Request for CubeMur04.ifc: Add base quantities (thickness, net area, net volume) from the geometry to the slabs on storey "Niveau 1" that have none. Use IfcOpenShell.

First a look at what the model holds.

```python
import ifcopenshell
import ifcopenshell.util.element
import ifcopenshell.util.unit

model = ifcopenshell.open("CubeMur04.ifc")
print(model.schema)
for unit_type in ("LENGTHUNIT", "AREAUNIT", "VOLUMEUNIT"):
    print(unit_type, ifcopenshell.util.unit.calculate_unit_scale(model, unit_type))
storey = next(s for s in model.by_type("IfcBuildingStorey") if s.Name == "Niveau 1")
slabs = [e for e in ifcopenshell.util.element.get_decomposition(storey) if e.is_a("IfcSlab")]
for e in sorted(slabs, key=lambda e: e.id()):
    print(e.id(), e.is_a(), e.Name, list(ifcopenshell.util.element.get_psets(e, qtos_only=True)), sep=" | ")
```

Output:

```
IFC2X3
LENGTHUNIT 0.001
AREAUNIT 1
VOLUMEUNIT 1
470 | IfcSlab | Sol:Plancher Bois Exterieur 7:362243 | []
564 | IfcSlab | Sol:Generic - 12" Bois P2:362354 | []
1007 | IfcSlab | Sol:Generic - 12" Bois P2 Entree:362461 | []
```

```python
import ifcopenshell
import ifcopenshell.api.pset
import ifcopenshell.geom
import ifcopenshell.util.element
import ifcopenshell.util.shape
import ifcopenshell.util.unit

model = ifcopenshell.open("CubeMur04.ifc")
unit_scale = ifcopenshell.util.unit.calculate_unit_scale(model)
area_scale = ifcopenshell.util.unit.calculate_unit_scale(model, "AREAUNIT")
volume_scale = ifcopenshell.util.unit.calculate_unit_scale(model, "VOLUMEUNIT")
settings = ifcopenshell.geom.settings()

storey = next(s for s in model.by_type("IfcBuildingStorey") if s.Name == "Niveau 1")
slabs = [e for e in ifcopenshell.util.element.get_decomposition(storey) if e.is_a("IfcSlab")]

for e in sorted(slabs, key=lambda e: e.id()):
    if ifcopenshell.util.element.get_psets(e, qtos_only=True, should_inherit=False):
        continue
    # Geometry comes back in metres, in the element's own axes.
    shape = ifcopenshell.geom.create_shape(settings, e)
    values = {
        "Width": ifcopenshell.util.shape.get_z(shape.geometry) / unit_scale,
        "NetArea": ifcopenshell.util.shape.get_footprint_area(shape.geometry) / area_scale,
        "NetVolume": ifcopenshell.util.shape.get_volume(shape.geometry) / volume_scale,
    }
    qto = ifcopenshell.api.pset.add_qto(model, product=e, name="BaseQuantities")
    ifcopenshell.api.pset.edit_qto(model, qto=qto, properties=values)
    print(e.id(), {k: round(v, 3) for k, v in values.items()})

model.write("CubeMur04_v2.ifc")
```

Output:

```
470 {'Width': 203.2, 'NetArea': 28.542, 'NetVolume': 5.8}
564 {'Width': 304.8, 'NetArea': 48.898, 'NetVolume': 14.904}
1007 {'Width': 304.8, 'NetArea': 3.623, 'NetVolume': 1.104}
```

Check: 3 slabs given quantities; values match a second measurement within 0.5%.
